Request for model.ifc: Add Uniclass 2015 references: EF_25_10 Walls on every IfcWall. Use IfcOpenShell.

First a look at what the model holds.

```python
import ifcopenshell

model = ifcopenshell.open("model.ifc")
print(model.schema)
print("classifications:", [c.Name for c in model.by_type("IfcClassification")])
for ifc_class in ("IfcDoor", "IfcRoof", "IfcStair", "IfcWall", "IfcWindow"):
    print(ifc_class, len(model.by_type(ifc_class)))
```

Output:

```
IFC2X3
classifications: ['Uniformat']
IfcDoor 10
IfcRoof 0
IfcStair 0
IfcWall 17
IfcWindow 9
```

```python
import ifcopenshell
import ifcopenshell.api.classification

model = ifcopenshell.open("model.ifc")

# IFC2X3 requires Source and Edition and has no link from the project to the system.
system = model.create_entity("IfcClassification", Source="NBS", Edition="2015", Name="Uniclass 2015")

codes = {
    "IfcWall": ("EF_25_10", "Walls"),
}
for ifc_class, (code, name) in codes.items():
    products = model.by_type(ifc_class)
    ifcopenshell.api.classification.add_reference(
        model, products=products, classification=system, identification=code, name=name
    )
    print(code, len(products))

model.write("model_rev.ifc")
```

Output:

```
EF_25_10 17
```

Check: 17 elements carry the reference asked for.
